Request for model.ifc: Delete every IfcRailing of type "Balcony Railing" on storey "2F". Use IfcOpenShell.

First a look at what the model holds.

```python
import ifcopenshell
import ifcopenshell.util.element

model = ifcopenshell.open("model.ifc")
print(model.schema)
storey = next(s for s in model.by_type("IfcBuildingStorey") if s.Name == "2F")
railings = [e for e in ifcopenshell.util.element.get_decomposition(storey) if e.is_a("IfcRailing")]
seen = {}
for e in railings:
    element_type = ifcopenshell.util.element.get_type(e)
    name = element_type.Name if element_type not in (None, e) else None
    seen[name] = seen.get(name, 0) + 1
for name, count in sorted(seen.items(), key=str):
    print(count, "x", name)
```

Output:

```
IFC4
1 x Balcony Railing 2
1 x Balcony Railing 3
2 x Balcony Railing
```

```python
import ifcopenshell
import ifcopenshell.api.root
import ifcopenshell.util.element

model = ifcopenshell.open("model.ifc")

storey = next(s for s in model.by_type("IfcBuildingStorey") if s.Name == "2F")
railings = [e for e in ifcopenshell.util.element.get_decomposition(storey) if e.is_a("IfcRailing")]
targets = [e for e in railings if (t := ifcopenshell.util.element.get_type(e)) not in (None, e) and t.Name == "Balcony Railing"]

for e in targets:
    ifcopenshell.api.root.remove_product(model, product=e)
print(len(targets), "removed")

model.write("model_v2.ifc")
```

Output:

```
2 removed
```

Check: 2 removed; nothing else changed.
